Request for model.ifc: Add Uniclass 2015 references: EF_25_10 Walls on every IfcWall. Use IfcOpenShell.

First a look at what the model holds.

```python
import ifcopenshell

model = ifcopenshell.open("model.ifc")
print(model.schema)
print("classifications:", [c.Name for c in model.by_type("IfcClassification")])
for ifc_class in ("IfcDoor", "IfcRoof", "IfcStair", "IfcWall", "IfcWindow"):
    print(ifc_class, len(model.by_type(ifc_class)))
```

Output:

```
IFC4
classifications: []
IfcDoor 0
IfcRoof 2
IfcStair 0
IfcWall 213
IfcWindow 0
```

```python
import ifcopenshell
import ifcopenshell.api.classification

model = ifcopenshell.open("model.ifc")

system = ifcopenshell.api.classification.add_classification(model, classification="Uniclass 2015")

codes = {
    "IfcWall": ("EF_25_10", "Walls"),
}
for ifc_class, (code, name) in codes.items():
    products = model.by_type(ifc_class)
    ifcopenshell.api.classification.add_reference(
        model, products=products, classification=system, identification=code, name=name
    )
    print(code, len(products))

model.write("model_v2.ifc")
```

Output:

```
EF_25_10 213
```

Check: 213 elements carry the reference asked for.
